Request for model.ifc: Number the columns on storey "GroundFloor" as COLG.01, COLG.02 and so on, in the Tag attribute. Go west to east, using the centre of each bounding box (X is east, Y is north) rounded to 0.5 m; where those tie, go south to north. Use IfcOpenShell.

First a look at what the model holds.

```python
import ifcopenshell
import ifcopenshell.util.element
import ifcopenshell.util.placement

model = ifcopenshell.open("model.ifc")
print(model.schema)
storey = next(s for s in model.by_type("IfcBuildingStorey") if s.Name == "GroundFloor")
columns = [e for e in ifcopenshell.util.element.get_decomposition(storey) if e.is_a("IfcColumn")]
for e in sorted(columns, key=lambda e: e.id()):
    origin = ifcopenshell.util.placement.get_local_placement(e.ObjectPlacement)[:3, 3]
    print(e.id(), e.Tag, e.Name, origin.round(2) + 0.0, sep=" | ")
```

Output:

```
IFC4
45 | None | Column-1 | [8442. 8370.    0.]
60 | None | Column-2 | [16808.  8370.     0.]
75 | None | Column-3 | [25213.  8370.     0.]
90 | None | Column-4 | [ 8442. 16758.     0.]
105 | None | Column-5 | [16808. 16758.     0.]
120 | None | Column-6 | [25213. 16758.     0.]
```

```python
import ifcopenshell
import ifcopenshell.geom
import ifcopenshell.util.element
import ifcopenshell.util.shape

model = ifcopenshell.open("model.ifc")
settings = ifcopenshell.geom.settings()
settings.set("use-world-coords", True)


def centre(element):
    shape = ifcopenshell.geom.create_shape(settings, element)
    return ifcopenshell.util.shape.get_bbox_centroid(shape.geometry)


storey = next(s for s in model.by_type("IfcBuildingStorey") if s.Name == "GroundFloor")
columns = [e for e in ifcopenshell.util.element.get_decomposition(storey) if e.is_a("IfcColumn")]

# Insertion points can sit at a corner or the storey origin, so sort by the geometry (in metres).
centres = {e: centre(e) for e in columns}
columns.sort(key=lambda e: (round(centres[e][0] / 0.5), centres[e][1]))

for i, e in enumerate(columns, start=1):
    number = f"COLG.{i:02d}"
    e.Tag = number
    print(e.id(), number)

model.write("model_v2.ifc")
```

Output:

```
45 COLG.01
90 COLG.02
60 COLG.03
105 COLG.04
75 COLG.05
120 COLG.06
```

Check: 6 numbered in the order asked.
